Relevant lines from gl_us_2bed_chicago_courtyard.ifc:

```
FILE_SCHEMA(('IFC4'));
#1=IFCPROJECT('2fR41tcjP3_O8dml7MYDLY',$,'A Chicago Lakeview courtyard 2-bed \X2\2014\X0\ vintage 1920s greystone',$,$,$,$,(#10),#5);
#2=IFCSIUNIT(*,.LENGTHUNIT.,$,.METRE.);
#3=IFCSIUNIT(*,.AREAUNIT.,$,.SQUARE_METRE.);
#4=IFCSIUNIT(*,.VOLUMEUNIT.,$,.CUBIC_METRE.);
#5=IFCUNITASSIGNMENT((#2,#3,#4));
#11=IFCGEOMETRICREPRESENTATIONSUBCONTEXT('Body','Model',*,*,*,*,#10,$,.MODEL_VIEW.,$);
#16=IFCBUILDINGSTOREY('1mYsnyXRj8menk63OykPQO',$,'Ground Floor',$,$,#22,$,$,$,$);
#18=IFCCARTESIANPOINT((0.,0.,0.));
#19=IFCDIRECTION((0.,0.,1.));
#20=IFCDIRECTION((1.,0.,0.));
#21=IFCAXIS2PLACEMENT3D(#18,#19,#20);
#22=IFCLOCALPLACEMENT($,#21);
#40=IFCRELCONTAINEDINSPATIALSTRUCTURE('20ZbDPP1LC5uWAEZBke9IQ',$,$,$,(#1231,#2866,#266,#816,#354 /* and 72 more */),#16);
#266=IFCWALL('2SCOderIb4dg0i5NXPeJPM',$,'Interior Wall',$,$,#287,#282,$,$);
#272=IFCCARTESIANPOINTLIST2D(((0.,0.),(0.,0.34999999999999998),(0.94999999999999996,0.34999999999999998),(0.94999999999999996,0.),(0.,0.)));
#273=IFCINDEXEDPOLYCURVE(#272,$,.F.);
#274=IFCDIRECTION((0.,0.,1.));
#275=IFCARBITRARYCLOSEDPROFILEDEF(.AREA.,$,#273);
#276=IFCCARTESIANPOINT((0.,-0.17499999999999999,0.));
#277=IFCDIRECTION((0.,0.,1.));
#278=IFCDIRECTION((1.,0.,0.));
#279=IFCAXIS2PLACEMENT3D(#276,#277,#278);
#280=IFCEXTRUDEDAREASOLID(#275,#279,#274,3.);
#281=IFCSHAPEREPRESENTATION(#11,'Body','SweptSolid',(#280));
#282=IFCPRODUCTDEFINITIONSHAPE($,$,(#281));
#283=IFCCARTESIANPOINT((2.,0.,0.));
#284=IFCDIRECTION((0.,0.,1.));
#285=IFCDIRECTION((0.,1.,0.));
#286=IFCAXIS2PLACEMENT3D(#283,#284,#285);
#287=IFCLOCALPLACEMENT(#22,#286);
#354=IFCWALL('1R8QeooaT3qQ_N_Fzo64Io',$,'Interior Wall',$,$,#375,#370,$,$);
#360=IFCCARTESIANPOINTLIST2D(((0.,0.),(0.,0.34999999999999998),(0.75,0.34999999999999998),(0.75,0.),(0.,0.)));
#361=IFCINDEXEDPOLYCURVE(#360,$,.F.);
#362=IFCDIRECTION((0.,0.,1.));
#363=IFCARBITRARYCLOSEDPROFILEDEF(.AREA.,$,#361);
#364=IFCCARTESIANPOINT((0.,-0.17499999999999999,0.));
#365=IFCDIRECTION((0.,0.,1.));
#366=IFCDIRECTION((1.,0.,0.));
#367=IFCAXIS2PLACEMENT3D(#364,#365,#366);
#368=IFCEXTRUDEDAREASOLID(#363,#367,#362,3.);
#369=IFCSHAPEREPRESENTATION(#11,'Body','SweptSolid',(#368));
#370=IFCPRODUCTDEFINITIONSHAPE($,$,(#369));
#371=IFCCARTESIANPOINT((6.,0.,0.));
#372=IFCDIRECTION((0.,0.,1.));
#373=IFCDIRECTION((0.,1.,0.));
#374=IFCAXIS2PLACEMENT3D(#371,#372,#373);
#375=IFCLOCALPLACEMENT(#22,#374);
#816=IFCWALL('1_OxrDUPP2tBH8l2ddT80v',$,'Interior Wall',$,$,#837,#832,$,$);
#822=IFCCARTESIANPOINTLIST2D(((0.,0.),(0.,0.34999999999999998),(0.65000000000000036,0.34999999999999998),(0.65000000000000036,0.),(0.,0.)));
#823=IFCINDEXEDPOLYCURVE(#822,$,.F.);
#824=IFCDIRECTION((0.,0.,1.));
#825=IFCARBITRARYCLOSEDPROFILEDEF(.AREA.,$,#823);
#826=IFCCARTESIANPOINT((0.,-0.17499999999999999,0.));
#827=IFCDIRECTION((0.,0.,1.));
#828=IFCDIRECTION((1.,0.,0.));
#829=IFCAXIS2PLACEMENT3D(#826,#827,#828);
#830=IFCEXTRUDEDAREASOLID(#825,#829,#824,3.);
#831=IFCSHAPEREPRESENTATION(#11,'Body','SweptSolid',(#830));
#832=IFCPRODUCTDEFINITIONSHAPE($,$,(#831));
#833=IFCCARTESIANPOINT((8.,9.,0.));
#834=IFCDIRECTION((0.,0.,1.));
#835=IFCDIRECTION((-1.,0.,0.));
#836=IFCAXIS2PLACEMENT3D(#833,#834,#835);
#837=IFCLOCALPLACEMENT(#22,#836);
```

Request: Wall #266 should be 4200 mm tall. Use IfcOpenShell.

```python
import ifcopenshell
import ifcopenshell.geom
import ifcopenshell.util.representation
import ifcopenshell.util.shape

model = ifcopenshell.open("gl_us_2bed_chicago_courtyard.ifc")
settings = ifcopenshell.geom.settings()


def volume(element):
    """Net volume in cubic metres, openings subtracted."""
    shape = ifcopenshell.geom.create_shape(settings, element)
    return ifcopenshell.util.shape.get_volume(shape.geometry)


wall = model.by_id(266)
before = volume(wall)

body = ifcopenshell.util.representation.get_representation(wall, "Model", "Body")
solid = body.Items[0]
old_height = solid.Depth
solid.Depth = 4.2
after = volume(wall)

print(f"height {old_height:g} -> {solid.Depth:g}, volume {before:.3f} -> {after:.3f} m3")

model.write("gl_us_2bed_chicago_courtyard-out.ifc")
```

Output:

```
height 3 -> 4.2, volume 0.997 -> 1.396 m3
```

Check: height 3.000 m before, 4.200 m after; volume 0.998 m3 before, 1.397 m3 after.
